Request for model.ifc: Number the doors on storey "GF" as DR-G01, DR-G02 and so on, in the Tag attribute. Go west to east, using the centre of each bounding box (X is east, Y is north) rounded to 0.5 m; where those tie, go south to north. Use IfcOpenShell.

First a look at what the model holds.

```python
import ifcopenshell
import ifcopenshell.util.element
import ifcopenshell.util.placement

model = ifcopenshell.open("model.ifc")
print(model.schema)
storey = next(s for s in model.by_type("IfcBuildingStorey") if s.Name == "GF")
doors = [e for e in ifcopenshell.util.element.get_decomposition(storey) if e.is_a("IfcDoor")]
for e in sorted(doors, key=lambda e: e.id()):
    origin = ifcopenshell.util.placement.get_local_placement(e.ObjectPlacement)[:3, 3]
    print(e.id(), e.Tag, e.Name, origin.round(2) + 0.0, sep=" | ")
```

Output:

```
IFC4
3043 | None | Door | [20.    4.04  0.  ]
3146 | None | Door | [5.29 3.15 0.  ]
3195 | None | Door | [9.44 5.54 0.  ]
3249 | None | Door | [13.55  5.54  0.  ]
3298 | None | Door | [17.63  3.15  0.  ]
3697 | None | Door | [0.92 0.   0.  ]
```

```python
import ifcopenshell
import ifcopenshell.geom
import ifcopenshell.util.element
import ifcopenshell.util.shape

model = ifcopenshell.open("model.ifc")
settings = ifcopenshell.geom.settings()
settings.set("use-world-coords", True)


def centre(element):
    shape = ifcopenshell.geom.create_shape(settings, element)
    return ifcopenshell.util.shape.get_bbox_centroid(shape.geometry)


storey = next(s for s in model.by_type("IfcBuildingStorey") if s.Name == "GF")
doors = [e for e in ifcopenshell.util.element.get_decomposition(storey) if e.is_a("IfcDoor")]

# Insertion points can sit at a corner or the storey origin, so sort by the geometry (in metres).
centres = {e: centre(e) for e in doors}
doors.sort(key=lambda e: (round(centres[e][0] / 0.5), centres[e][1]))

for i, e in enumerate(doors, start=1):
    number = f"DR-G{i:02d}"
    e.Tag = number
    print(e.id(), number)

model.write("model_v2.ifc")
```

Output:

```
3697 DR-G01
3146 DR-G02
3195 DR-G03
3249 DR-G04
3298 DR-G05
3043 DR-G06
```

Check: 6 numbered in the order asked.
